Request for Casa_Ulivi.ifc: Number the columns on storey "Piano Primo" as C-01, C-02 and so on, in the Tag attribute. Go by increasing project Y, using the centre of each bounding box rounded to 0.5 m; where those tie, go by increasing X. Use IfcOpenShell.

First a look at what the model holds.

```python
import ifcopenshell
import ifcopenshell.util.element
import ifcopenshell.util.placement

model = ifcopenshell.open("Casa_Ulivi.ifc")
print(model.schema)
storey = next(s for s in model.by_type("IfcBuildingStorey") if s.Name == "Piano Primo")
columns = [e for e in ifcopenshell.util.element.get_decomposition(storey) if e.is_a("IfcColumn")]
for e in sorted(columns, key=lambda e: e.id()):
    origin = ifcopenshell.util.placement.get_local_placement(e.ObjectPlacement)[:3, 3]
    print(e.id(), e.Tag, e.Name, origin.round(2) + 0.0, sep=" | ")
```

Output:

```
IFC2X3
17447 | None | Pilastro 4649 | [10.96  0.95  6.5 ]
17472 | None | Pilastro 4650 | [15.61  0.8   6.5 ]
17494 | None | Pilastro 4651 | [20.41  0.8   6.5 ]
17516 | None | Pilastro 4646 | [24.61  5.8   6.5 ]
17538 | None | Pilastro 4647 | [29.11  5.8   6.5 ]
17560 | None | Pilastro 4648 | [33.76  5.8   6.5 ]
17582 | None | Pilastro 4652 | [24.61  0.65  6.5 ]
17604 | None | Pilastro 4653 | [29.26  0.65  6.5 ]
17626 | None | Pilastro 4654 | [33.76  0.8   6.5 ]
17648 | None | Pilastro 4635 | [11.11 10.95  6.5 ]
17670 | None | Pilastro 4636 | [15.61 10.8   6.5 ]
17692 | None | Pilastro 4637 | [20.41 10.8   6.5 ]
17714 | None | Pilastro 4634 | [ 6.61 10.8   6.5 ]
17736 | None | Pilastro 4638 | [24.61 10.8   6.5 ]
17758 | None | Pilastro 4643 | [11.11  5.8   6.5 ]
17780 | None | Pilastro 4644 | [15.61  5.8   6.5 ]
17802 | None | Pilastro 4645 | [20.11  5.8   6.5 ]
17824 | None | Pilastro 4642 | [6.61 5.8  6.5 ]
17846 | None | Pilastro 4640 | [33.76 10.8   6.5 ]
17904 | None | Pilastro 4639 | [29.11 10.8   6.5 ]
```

```python
import ifcopenshell
import ifcopenshell.geom
import ifcopenshell.util.element
import ifcopenshell.util.shape

model = ifcopenshell.open("Casa_Ulivi.ifc")
settings = ifcopenshell.geom.settings()
settings.set("use-world-coords", True)


def centre(element):
    shape = ifcopenshell.geom.create_shape(settings, element)
    return ifcopenshell.util.shape.get_bbox_centroid(shape.geometry)


storey = next(s for s in model.by_type("IfcBuildingStorey") if s.Name == "Piano Primo")
columns = [e for e in ifcopenshell.util.element.get_decomposition(storey) if e.is_a("IfcColumn")]

# Insertion points can sit at a corner or the storey origin, so sort by the geometry (in metres).
centres = {e: centre(e) for e in columns}
columns.sort(key=lambda e: (round(centres[e][1] / 0.5), centres[e][0]))

for i, e in enumerate(columns, start=1):
    number = f"C-{i:02d}"
    e.Tag = number
    print(e.id(), number)

model.write("Casa_Ulivi_v2.ifc")
```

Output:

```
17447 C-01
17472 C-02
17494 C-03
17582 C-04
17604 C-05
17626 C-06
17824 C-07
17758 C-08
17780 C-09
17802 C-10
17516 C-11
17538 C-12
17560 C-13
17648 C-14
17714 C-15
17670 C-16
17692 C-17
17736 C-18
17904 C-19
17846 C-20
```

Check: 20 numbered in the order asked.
